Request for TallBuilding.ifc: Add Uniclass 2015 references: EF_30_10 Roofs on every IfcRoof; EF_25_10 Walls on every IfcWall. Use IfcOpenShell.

First a look at what the model holds.

```python
import ifcopenshell

model = ifcopenshell.open("TallBuilding.ifc")
print(model.schema)
print("classifications:", [c.Name for c in model.by_type("IfcClassification")])
for ifc_class in ("IfcDoor", "IfcRoof", "IfcStair", "IfcWall", "IfcWindow"):
    print(ifc_class, len(model.by_type(ifc_class)))
```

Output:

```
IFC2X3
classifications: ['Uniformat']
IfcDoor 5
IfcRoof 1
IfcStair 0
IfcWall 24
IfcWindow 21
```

```python
import ifcopenshell
import ifcopenshell.api.classification

model = ifcopenshell.open("TallBuilding.ifc")

# IFC2X3 requires Source and Edition and has no link from the project to the system.
system = model.create_entity("IfcClassification", Source="NBS", Edition="2015", Name="Uniclass 2015")

codes = {
    "IfcRoof": ("EF_30_10", "Roofs"),
    "IfcWall": ("EF_25_10", "Walls"),
}
for ifc_class, (code, name) in codes.items():
    products = model.by_type(ifc_class)
    ifcopenshell.api.classification.add_reference(
        model, products=products, classification=system, identification=code, name=name
    )
    print(code, len(products))

model.write("TallBuilding_edited.ifc")
```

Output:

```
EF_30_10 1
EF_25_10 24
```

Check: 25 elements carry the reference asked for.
